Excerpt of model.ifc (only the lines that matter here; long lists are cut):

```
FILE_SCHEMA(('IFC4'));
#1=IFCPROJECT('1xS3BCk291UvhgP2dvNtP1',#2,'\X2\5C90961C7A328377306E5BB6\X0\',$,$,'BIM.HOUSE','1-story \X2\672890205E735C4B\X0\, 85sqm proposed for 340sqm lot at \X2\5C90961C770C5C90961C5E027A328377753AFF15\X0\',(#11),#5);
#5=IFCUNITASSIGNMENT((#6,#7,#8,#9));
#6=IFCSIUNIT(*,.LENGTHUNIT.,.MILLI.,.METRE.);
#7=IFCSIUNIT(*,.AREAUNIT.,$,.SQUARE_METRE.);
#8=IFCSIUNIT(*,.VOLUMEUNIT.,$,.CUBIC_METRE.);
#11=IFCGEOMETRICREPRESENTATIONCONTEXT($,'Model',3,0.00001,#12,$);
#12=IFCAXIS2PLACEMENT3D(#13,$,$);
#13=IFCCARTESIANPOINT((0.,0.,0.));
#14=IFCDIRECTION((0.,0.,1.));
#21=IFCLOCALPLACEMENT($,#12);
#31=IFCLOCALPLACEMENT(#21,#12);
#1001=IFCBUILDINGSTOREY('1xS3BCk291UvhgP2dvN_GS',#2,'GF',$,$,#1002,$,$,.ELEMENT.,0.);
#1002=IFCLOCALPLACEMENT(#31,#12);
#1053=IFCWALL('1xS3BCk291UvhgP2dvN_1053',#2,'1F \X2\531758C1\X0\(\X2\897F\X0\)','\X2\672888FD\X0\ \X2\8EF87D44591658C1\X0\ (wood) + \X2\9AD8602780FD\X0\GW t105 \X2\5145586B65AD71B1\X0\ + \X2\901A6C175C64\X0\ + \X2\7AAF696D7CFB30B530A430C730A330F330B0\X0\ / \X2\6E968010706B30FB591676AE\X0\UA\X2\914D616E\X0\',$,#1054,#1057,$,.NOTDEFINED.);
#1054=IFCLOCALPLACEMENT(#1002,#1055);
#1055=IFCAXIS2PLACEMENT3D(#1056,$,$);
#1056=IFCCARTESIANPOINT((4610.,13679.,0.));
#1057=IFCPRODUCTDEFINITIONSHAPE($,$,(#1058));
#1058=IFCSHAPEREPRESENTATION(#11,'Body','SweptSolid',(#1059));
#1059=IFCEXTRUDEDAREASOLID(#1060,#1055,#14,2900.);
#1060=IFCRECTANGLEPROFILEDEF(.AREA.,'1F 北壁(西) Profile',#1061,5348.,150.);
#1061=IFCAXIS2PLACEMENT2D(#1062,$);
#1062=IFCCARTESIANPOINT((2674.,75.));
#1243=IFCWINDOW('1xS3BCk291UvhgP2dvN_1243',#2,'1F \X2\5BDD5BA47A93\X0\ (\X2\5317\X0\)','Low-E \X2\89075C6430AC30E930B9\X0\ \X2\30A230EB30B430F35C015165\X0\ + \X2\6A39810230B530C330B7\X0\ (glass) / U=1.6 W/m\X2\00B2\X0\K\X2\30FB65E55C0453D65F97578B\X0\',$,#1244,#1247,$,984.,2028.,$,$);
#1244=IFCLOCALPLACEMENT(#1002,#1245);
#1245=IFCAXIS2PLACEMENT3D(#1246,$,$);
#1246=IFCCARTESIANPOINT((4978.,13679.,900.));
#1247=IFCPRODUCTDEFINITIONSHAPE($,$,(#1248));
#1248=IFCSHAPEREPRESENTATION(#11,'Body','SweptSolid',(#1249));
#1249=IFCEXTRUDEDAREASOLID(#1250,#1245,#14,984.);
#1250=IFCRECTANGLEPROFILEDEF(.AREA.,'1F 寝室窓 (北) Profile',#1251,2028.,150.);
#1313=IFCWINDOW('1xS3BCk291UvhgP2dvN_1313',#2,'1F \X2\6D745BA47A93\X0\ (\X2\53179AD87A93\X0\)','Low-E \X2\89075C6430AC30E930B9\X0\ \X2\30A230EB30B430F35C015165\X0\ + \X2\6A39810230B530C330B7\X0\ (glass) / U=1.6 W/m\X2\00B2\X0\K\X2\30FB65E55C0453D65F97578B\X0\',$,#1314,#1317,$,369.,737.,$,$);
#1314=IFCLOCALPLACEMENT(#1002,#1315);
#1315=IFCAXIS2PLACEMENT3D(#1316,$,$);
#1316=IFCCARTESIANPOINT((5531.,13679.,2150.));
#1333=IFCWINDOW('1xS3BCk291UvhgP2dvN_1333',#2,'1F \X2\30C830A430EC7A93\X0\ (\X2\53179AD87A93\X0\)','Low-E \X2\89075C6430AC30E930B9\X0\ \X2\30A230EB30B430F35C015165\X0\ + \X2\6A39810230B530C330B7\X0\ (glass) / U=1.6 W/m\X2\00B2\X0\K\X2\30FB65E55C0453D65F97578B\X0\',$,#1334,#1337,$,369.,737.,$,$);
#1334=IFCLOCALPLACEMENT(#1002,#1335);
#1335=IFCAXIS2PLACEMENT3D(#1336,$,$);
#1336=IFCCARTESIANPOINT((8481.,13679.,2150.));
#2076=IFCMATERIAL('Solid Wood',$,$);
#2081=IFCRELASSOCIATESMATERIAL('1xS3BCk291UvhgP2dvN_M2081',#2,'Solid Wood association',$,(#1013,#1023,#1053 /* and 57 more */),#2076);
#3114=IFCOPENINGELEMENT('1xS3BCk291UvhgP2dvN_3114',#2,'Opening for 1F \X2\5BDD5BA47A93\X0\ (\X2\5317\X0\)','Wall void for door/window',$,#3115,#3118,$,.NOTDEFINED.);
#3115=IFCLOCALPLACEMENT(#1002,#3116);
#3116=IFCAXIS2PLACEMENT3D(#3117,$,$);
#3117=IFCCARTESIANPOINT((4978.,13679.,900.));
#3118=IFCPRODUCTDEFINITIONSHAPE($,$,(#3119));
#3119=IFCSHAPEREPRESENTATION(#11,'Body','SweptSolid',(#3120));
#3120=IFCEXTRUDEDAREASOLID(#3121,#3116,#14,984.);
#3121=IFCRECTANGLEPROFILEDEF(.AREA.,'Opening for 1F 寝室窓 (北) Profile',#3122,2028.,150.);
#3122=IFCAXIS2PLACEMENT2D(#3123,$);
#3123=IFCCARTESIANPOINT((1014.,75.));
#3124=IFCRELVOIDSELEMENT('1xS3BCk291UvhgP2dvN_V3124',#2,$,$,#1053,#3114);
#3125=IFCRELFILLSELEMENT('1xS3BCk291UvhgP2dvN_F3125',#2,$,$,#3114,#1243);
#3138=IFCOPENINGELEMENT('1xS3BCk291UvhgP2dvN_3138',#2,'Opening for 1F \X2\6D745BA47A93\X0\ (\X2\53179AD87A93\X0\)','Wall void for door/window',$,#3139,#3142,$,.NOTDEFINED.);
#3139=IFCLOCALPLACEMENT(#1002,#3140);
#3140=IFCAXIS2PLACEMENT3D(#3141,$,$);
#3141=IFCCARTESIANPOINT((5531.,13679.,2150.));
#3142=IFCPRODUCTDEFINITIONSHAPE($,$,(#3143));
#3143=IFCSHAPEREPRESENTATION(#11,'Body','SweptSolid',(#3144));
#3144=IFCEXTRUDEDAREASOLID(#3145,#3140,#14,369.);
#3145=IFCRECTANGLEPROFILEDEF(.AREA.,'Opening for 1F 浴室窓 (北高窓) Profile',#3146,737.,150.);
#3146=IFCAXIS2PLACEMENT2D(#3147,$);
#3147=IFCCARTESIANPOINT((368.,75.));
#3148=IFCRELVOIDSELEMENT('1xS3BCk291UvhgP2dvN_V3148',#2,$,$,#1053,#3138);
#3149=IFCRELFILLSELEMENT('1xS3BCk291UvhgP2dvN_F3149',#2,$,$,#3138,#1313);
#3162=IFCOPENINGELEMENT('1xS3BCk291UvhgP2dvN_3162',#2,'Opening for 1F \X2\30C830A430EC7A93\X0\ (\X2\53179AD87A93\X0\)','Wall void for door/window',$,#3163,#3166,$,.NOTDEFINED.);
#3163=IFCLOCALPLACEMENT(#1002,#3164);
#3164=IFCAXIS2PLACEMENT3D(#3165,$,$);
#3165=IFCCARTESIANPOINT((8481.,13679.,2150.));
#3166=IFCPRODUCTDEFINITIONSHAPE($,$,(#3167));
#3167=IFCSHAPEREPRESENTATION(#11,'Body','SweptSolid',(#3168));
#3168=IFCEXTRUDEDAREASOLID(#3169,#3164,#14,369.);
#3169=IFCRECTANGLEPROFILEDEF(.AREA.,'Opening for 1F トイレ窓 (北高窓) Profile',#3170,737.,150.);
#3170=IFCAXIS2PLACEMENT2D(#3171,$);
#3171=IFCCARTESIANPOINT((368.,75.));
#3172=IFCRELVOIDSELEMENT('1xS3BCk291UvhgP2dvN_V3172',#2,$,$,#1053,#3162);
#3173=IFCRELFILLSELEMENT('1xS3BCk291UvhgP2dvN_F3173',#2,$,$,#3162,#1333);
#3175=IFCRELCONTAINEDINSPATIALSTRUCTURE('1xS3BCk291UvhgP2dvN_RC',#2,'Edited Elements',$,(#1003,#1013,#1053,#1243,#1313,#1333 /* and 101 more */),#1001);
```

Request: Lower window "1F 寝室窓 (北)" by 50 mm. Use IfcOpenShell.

```python
import numpy as np
import ifcopenshell
import ifcopenshell.api.geometry
import ifcopenshell.util.placement
import ifcopenshell.util.unit

model = ifcopenshell.open("model.ifc")
unit_scale = ifcopenshell.util.unit.calculate_unit_scale(model)

window = model.by_id(1243)
opening = window.FillsVoids[0].RelatingOpeningElement
dz = -0.05 / unit_scale

shift = np.array([0.0, 0.0, dz])
# The window is not placed relative to its opening, so move both.
for product in (opening, window):
    matrix = ifcopenshell.util.placement.get_local_placement(product.ObjectPlacement)
    matrix[:3, 3] += shift
    ifcopenshell.api.geometry.edit_object_placement(model, product=product, matrix=matrix, is_si=False)

print(f"moved by {dz * unit_scale:+.3f} m")

model.write("model_rev.ifc")
```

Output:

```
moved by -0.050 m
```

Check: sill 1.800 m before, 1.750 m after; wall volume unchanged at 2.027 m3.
